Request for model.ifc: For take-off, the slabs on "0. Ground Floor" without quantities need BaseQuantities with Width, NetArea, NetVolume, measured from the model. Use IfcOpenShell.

First a look at what the model holds.

```python
import ifcopenshell
import ifcopenshell.util.element
import ifcopenshell.util.unit

model = ifcopenshell.open("model.ifc")
print(model.schema)
for unit_type in ("LENGTHUNIT", "AREAUNIT", "VOLUMEUNIT"):
    print(unit_type, ifcopenshell.util.unit.calculate_unit_scale(model, unit_type))
storey = next(s for s in model.by_type("IfcBuildingStorey") if s.Name == "0. Ground Floor")
slabs = [e for e in ifcopenshell.util.element.get_decomposition(storey) if e.is_a("IfcSlab")]
for e in sorted(slabs, key=lambda e: e.id()):
    print(e.id(), e.is_a(), e.Name, list(ifcopenshell.util.element.get_psets(e, qtos_only=True)), sep=" | ")
```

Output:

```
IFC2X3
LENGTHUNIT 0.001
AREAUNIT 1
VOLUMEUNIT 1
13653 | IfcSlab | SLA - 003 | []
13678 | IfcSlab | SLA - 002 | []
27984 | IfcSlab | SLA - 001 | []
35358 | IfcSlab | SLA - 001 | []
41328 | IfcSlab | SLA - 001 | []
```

```python
import ifcopenshell
import ifcopenshell.api.pset
import ifcopenshell.geom
import ifcopenshell.util.element
import ifcopenshell.util.shape
import ifcopenshell.util.unit

model = ifcopenshell.open("model.ifc")
unit_scale = ifcopenshell.util.unit.calculate_unit_scale(model)
area_scale = ifcopenshell.util.unit.calculate_unit_scale(model, "AREAUNIT")
volume_scale = ifcopenshell.util.unit.calculate_unit_scale(model, "VOLUMEUNIT")
settings = ifcopenshell.geom.settings()

storey = next(s for s in model.by_type("IfcBuildingStorey") if s.Name == "0. Ground Floor")
slabs = [e for e in ifcopenshell.util.element.get_decomposition(storey) if e.is_a("IfcSlab")]

for e in sorted(slabs, key=lambda e: e.id()):
    if ifcopenshell.util.element.get_psets(e, qtos_only=True, should_inherit=False):
        continue
    # Geometry comes back in metres, in the element's own axes.
    shape = ifcopenshell.geom.create_shape(settings, e)
    values = {
        "Width": ifcopenshell.util.shape.get_z(shape.geometry) / unit_scale,
        "NetArea": ifcopenshell.util.shape.get_footprint_area(shape.geometry) / area_scale,
        "NetVolume": ifcopenshell.util.shape.get_volume(shape.geometry) / volume_scale,
    }
    qto = ifcopenshell.api.pset.add_qto(model, product=e, name="BaseQuantities")
    ifcopenshell.api.pset.edit_qto(model, qto=qto, properties=values)
    print(e.id(), {k: round(v, 3) for k, v in values.items()})

model.write("model-out.ifc")
```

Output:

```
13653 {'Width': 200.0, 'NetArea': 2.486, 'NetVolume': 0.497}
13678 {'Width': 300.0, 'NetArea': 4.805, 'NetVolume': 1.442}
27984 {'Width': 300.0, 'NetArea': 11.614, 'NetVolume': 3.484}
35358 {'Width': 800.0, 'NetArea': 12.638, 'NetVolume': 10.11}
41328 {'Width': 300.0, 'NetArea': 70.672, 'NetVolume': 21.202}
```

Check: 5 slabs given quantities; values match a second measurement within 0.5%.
